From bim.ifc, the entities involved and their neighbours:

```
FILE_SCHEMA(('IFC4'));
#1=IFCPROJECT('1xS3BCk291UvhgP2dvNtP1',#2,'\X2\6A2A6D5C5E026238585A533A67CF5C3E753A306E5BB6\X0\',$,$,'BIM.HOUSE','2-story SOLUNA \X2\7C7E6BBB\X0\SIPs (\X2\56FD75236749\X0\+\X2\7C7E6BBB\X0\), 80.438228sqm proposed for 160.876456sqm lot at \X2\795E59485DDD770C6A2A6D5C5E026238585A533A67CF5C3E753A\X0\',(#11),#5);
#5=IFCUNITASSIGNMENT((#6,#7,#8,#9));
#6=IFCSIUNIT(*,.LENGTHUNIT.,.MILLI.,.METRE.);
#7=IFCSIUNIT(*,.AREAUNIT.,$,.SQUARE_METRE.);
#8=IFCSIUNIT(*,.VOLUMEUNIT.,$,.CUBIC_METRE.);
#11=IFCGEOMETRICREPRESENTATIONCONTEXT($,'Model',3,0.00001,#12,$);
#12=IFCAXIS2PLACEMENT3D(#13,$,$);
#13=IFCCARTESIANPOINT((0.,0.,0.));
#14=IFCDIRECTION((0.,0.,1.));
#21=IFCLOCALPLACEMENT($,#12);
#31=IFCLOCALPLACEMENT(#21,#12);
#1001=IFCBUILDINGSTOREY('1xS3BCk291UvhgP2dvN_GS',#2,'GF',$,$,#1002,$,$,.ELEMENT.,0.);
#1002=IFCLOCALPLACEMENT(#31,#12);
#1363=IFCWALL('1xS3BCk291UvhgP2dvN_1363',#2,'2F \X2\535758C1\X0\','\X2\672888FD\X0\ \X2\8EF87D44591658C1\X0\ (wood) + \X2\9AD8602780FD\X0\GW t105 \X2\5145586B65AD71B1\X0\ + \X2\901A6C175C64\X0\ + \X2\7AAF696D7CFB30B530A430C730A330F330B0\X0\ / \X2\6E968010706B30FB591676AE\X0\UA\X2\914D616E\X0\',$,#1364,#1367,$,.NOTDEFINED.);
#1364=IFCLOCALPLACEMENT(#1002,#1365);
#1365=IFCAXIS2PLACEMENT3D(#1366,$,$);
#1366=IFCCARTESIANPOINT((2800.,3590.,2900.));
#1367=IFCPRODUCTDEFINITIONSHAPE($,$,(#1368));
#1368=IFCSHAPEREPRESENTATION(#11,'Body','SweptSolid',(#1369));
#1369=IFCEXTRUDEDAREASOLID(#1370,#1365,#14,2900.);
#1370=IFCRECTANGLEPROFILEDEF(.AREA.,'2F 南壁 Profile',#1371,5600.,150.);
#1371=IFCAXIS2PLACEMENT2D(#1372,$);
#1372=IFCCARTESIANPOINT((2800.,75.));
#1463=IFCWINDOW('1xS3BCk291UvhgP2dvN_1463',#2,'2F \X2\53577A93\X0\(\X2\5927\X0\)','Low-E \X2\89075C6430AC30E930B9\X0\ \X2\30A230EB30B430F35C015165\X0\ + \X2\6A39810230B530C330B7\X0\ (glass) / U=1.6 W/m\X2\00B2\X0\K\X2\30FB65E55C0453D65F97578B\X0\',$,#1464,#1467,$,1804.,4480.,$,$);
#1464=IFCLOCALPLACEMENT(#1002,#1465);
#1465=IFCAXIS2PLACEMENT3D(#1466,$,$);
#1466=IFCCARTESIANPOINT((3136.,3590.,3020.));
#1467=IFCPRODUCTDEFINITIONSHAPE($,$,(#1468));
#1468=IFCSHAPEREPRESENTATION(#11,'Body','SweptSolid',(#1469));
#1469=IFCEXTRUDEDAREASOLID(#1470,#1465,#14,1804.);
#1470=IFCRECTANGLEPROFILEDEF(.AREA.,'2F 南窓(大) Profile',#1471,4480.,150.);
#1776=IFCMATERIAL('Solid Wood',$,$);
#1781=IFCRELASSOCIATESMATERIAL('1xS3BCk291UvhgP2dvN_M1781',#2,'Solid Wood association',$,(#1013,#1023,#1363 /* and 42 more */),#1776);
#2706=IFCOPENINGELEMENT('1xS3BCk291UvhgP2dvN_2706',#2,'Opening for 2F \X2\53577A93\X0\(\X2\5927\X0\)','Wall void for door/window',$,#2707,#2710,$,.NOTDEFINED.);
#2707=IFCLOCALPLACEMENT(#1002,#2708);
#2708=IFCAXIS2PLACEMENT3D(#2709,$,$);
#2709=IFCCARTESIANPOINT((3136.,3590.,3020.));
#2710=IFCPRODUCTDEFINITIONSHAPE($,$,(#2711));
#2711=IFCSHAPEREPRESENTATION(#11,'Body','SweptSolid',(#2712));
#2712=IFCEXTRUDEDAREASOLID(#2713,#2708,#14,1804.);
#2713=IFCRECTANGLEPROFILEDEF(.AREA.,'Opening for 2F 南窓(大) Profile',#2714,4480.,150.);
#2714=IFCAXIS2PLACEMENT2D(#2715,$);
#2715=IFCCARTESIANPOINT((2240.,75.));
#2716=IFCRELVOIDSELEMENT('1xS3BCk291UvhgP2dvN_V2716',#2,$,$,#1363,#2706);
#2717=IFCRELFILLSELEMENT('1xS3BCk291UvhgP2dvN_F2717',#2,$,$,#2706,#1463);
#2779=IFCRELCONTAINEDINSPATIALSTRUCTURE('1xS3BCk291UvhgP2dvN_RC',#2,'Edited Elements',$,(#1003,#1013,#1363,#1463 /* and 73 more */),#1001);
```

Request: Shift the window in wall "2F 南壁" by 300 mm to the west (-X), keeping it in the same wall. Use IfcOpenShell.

```python
import ifcopenshell
import ifcopenshell.api.geometry
import ifcopenshell.util.placement

model = ifcopenshell.open("bim.ifc")

window = model.by_guid("1xS3BCk291UvhgP2dvN_1463")
opening = window.FillsVoids[0].RelatingOpeningElement
wall = opening.VoidsElements[0].RelatingBuildingElement

wall_matrix = ifcopenshell.util.placement.get_local_placement(wall.ObjectPlacement)
shift = wall_matrix[:3, 0] * -300.0
before = ifcopenshell.util.placement.get_local_placement(window.ObjectPlacement)[:3, 3].copy()

# The window is not placed relative to its opening, so move both.
for product in (opening, window):
    matrix = ifcopenshell.util.placement.get_local_placement(product.ObjectPlacement)
    matrix[:3, 3] += shift
    ifcopenshell.api.geometry.edit_object_placement(model, product=product, matrix=matrix, is_si=False)

after = ifcopenshell.util.placement.get_local_placement(window.ObjectPlacement)[:3, 3]
print("window moved by", (after - before).round(3) + 0.0)

model.write("bim_updated.ifc")
```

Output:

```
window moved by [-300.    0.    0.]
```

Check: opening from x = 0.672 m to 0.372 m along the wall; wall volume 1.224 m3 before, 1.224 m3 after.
